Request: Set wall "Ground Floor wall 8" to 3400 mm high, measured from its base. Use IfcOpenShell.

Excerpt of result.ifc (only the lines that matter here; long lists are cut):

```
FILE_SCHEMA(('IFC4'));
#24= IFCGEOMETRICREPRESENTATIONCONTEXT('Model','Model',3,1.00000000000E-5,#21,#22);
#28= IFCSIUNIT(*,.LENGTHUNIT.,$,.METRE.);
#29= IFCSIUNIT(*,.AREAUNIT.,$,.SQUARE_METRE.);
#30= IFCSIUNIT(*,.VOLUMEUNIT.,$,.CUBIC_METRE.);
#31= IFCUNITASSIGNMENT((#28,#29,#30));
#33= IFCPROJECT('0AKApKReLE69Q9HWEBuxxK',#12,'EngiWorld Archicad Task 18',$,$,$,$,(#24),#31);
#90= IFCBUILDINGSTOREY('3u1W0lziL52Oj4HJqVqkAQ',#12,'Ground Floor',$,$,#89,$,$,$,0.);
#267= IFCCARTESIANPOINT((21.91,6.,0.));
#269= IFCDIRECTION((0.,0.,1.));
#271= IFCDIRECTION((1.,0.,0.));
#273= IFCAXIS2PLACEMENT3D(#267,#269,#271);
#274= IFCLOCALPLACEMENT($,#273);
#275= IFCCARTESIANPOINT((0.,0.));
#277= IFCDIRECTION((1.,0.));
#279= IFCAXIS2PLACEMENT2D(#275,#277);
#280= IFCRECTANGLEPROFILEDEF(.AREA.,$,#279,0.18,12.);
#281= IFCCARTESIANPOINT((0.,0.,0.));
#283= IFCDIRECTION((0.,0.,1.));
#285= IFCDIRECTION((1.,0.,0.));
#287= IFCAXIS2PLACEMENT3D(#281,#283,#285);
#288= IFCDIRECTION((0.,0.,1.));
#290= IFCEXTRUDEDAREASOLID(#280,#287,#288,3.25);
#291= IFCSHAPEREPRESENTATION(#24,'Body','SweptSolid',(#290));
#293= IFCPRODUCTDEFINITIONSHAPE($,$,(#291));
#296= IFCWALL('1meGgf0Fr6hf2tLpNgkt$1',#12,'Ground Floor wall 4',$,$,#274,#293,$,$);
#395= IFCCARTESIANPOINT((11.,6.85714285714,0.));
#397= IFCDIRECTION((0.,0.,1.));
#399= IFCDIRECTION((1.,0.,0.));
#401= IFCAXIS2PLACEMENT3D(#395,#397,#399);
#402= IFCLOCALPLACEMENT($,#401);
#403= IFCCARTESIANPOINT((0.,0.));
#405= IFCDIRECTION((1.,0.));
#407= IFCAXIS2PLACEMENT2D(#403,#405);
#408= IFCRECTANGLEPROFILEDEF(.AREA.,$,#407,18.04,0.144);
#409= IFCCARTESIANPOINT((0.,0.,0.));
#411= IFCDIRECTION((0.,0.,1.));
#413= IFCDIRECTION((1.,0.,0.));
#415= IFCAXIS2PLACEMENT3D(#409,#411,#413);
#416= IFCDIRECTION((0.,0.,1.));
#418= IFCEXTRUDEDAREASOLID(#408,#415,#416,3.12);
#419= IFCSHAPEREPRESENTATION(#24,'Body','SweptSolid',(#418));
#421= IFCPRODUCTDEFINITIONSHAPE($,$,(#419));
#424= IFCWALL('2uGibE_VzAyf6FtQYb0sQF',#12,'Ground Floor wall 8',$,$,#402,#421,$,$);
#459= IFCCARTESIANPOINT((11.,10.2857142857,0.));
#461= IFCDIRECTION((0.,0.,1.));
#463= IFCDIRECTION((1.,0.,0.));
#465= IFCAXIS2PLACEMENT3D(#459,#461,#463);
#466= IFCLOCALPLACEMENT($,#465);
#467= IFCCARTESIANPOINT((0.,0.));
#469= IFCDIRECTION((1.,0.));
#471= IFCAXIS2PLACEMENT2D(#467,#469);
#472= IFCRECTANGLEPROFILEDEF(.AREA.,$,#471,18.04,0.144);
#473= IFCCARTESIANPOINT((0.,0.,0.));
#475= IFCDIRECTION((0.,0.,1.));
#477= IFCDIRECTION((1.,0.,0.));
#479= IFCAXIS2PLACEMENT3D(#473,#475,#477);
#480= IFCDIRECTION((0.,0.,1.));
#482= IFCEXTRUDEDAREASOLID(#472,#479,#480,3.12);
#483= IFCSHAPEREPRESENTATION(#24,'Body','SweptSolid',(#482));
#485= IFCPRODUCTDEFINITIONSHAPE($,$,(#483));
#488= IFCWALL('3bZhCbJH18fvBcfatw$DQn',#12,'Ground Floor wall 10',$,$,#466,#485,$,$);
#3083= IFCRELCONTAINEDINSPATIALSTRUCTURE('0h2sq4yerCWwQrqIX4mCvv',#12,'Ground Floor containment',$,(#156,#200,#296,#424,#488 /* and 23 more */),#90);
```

```python
import ifcopenshell
import ifcopenshell.geom
import ifcopenshell.util.shape

model = ifcopenshell.open("result.ifc")
settings = ifcopenshell.geom.settings()


def volume(element):
    """Net volume in cubic metres, openings subtracted."""
    shape = ifcopenshell.geom.create_shape(settings, element)
    return ifcopenshell.util.shape.get_volume(shape.geometry)


wall = model.by_guid("2uGibE_VzAyf6FtQYb0sQF")
before = volume(wall)

body = next(r for r in wall.Representation.Representations if r.RepresentationIdentifier == "Body")
solid = body.Items[0]
old_height = solid.Depth
solid.Depth = 3.4
after = volume(wall)

print(f"height {old_height:g} -> {solid.Depth:g}, volume {before:.3f} -> {after:.3f} m3")

model.write("result-out.ifc")
```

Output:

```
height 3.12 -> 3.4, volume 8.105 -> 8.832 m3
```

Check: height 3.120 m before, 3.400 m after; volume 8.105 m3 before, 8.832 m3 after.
